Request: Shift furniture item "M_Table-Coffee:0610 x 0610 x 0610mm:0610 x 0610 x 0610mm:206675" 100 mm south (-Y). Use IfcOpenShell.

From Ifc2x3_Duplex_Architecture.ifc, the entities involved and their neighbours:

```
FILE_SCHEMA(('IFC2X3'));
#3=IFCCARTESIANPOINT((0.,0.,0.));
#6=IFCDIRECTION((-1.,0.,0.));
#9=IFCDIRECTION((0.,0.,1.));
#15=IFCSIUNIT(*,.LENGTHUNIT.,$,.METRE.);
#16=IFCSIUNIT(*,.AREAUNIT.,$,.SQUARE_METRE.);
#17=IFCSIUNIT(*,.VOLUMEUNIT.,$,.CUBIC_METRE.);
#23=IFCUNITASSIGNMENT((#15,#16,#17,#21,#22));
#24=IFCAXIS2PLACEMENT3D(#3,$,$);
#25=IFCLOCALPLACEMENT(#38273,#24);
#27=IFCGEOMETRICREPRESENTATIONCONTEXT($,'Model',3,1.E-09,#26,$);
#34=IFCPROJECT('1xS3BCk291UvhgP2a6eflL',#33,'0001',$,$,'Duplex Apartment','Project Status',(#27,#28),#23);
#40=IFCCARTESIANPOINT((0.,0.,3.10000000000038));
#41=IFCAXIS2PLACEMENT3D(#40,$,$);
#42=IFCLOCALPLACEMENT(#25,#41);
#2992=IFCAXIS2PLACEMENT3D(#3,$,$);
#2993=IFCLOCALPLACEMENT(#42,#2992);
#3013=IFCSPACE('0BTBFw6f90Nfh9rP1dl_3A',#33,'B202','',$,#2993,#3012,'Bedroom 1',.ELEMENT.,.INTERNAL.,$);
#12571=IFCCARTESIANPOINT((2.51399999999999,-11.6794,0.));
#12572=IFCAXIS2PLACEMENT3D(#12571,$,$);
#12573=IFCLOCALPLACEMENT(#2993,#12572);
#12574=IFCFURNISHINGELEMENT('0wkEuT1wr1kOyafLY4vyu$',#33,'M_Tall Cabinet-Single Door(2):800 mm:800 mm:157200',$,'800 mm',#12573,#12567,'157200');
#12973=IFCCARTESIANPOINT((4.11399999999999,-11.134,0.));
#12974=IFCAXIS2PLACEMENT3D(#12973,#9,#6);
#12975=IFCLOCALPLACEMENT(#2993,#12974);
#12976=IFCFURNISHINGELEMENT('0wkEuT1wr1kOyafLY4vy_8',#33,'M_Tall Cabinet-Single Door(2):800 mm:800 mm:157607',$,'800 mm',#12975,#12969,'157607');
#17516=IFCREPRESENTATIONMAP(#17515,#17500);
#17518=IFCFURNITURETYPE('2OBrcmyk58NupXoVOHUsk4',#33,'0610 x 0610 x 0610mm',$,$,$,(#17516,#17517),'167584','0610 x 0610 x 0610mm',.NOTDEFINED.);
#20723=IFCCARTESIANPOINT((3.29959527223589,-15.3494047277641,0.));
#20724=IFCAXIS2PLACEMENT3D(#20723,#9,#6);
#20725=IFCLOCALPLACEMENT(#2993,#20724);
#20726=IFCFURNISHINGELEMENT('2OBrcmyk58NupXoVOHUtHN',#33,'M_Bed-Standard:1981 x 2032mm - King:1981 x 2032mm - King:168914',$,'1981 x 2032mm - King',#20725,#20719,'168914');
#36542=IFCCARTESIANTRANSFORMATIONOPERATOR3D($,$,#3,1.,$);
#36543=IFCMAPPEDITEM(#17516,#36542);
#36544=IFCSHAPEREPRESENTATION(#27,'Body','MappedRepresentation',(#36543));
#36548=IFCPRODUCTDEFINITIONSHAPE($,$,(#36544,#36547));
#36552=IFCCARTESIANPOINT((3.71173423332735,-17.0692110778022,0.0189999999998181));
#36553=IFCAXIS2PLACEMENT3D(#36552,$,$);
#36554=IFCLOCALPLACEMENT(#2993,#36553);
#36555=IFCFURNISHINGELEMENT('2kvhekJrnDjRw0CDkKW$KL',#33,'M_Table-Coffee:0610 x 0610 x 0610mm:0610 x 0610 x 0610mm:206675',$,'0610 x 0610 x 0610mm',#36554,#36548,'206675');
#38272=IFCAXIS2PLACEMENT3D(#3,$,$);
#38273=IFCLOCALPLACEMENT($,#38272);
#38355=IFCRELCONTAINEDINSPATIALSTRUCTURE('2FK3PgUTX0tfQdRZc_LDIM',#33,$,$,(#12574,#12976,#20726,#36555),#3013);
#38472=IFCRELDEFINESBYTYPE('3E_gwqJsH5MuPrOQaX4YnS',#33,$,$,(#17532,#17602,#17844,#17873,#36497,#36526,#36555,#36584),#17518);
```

```python
import ifcopenshell
import ifcopenshell.api.geometry
import ifcopenshell.util.placement

model = ifcopenshell.open("Ifc2x3_Duplex_Architecture.ifc")

item = model.by_id(36555)
matrix = ifcopenshell.util.placement.get_local_placement(item.ObjectPlacement)
matrix[1, 3] -= 0.1
ifcopenshell.api.geometry.edit_object_placement(model, product=item, matrix=matrix, is_si=False)

print(ifcopenshell.util.placement.get_local_placement(item.ObjectPlacement).round(3) + 0.0)

model.write("Ifc2x3_Duplex_Architecture_rev.ifc")
```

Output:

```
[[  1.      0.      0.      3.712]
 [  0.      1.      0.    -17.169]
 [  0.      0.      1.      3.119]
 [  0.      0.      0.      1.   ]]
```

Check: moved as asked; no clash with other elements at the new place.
